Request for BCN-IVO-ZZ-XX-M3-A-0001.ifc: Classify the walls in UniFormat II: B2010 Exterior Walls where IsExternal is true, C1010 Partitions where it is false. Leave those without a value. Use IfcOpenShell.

First a look at what the model holds.

```python
import ifcopenshell
import ifcopenshell.util.element

model = ifcopenshell.open("BCN-IVO-ZZ-XX-M3-A-0001.ifc")
print(model.schema)
print("classifications:", [c.Name for c in model.by_type("IfcClassification")])
values = [ifcopenshell.util.element.get_pset(e, "Pset_WallCommon", "IsExternal") for e in model.by_type("IfcWall")]
for value in (True, False, None):
    print("IsExternal", value, values.count(value))
```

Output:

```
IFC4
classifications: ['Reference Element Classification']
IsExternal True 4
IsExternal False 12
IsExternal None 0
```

```python
import ifcopenshell
import ifcopenshell.api.classification
import ifcopenshell.util.element

model = ifcopenshell.open("BCN-IVO-ZZ-XX-M3-A-0001.ifc")

system = ifcopenshell.api.classification.add_classification(model, classification="UniFormat II")

walls = model.by_type("IfcWall")
external = {e: ifcopenshell.util.element.get_pset(e, "Pset_WallCommon", "IsExternal") for e in walls}
for flag, code, name in ((True, "B2010", "Exterior Walls"), (False, "C1010", "Partitions")):
    products = [e for e in walls if external[e] is flag]
    ifcopenshell.api.classification.add_reference(
        model, products=products, classification=system, identification=code, name=name
    )
    print(code, len(products))

model.write("BCN-IVO-ZZ-XX-M3-A-0001_rev.ifc")
```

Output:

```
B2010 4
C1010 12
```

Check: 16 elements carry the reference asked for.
